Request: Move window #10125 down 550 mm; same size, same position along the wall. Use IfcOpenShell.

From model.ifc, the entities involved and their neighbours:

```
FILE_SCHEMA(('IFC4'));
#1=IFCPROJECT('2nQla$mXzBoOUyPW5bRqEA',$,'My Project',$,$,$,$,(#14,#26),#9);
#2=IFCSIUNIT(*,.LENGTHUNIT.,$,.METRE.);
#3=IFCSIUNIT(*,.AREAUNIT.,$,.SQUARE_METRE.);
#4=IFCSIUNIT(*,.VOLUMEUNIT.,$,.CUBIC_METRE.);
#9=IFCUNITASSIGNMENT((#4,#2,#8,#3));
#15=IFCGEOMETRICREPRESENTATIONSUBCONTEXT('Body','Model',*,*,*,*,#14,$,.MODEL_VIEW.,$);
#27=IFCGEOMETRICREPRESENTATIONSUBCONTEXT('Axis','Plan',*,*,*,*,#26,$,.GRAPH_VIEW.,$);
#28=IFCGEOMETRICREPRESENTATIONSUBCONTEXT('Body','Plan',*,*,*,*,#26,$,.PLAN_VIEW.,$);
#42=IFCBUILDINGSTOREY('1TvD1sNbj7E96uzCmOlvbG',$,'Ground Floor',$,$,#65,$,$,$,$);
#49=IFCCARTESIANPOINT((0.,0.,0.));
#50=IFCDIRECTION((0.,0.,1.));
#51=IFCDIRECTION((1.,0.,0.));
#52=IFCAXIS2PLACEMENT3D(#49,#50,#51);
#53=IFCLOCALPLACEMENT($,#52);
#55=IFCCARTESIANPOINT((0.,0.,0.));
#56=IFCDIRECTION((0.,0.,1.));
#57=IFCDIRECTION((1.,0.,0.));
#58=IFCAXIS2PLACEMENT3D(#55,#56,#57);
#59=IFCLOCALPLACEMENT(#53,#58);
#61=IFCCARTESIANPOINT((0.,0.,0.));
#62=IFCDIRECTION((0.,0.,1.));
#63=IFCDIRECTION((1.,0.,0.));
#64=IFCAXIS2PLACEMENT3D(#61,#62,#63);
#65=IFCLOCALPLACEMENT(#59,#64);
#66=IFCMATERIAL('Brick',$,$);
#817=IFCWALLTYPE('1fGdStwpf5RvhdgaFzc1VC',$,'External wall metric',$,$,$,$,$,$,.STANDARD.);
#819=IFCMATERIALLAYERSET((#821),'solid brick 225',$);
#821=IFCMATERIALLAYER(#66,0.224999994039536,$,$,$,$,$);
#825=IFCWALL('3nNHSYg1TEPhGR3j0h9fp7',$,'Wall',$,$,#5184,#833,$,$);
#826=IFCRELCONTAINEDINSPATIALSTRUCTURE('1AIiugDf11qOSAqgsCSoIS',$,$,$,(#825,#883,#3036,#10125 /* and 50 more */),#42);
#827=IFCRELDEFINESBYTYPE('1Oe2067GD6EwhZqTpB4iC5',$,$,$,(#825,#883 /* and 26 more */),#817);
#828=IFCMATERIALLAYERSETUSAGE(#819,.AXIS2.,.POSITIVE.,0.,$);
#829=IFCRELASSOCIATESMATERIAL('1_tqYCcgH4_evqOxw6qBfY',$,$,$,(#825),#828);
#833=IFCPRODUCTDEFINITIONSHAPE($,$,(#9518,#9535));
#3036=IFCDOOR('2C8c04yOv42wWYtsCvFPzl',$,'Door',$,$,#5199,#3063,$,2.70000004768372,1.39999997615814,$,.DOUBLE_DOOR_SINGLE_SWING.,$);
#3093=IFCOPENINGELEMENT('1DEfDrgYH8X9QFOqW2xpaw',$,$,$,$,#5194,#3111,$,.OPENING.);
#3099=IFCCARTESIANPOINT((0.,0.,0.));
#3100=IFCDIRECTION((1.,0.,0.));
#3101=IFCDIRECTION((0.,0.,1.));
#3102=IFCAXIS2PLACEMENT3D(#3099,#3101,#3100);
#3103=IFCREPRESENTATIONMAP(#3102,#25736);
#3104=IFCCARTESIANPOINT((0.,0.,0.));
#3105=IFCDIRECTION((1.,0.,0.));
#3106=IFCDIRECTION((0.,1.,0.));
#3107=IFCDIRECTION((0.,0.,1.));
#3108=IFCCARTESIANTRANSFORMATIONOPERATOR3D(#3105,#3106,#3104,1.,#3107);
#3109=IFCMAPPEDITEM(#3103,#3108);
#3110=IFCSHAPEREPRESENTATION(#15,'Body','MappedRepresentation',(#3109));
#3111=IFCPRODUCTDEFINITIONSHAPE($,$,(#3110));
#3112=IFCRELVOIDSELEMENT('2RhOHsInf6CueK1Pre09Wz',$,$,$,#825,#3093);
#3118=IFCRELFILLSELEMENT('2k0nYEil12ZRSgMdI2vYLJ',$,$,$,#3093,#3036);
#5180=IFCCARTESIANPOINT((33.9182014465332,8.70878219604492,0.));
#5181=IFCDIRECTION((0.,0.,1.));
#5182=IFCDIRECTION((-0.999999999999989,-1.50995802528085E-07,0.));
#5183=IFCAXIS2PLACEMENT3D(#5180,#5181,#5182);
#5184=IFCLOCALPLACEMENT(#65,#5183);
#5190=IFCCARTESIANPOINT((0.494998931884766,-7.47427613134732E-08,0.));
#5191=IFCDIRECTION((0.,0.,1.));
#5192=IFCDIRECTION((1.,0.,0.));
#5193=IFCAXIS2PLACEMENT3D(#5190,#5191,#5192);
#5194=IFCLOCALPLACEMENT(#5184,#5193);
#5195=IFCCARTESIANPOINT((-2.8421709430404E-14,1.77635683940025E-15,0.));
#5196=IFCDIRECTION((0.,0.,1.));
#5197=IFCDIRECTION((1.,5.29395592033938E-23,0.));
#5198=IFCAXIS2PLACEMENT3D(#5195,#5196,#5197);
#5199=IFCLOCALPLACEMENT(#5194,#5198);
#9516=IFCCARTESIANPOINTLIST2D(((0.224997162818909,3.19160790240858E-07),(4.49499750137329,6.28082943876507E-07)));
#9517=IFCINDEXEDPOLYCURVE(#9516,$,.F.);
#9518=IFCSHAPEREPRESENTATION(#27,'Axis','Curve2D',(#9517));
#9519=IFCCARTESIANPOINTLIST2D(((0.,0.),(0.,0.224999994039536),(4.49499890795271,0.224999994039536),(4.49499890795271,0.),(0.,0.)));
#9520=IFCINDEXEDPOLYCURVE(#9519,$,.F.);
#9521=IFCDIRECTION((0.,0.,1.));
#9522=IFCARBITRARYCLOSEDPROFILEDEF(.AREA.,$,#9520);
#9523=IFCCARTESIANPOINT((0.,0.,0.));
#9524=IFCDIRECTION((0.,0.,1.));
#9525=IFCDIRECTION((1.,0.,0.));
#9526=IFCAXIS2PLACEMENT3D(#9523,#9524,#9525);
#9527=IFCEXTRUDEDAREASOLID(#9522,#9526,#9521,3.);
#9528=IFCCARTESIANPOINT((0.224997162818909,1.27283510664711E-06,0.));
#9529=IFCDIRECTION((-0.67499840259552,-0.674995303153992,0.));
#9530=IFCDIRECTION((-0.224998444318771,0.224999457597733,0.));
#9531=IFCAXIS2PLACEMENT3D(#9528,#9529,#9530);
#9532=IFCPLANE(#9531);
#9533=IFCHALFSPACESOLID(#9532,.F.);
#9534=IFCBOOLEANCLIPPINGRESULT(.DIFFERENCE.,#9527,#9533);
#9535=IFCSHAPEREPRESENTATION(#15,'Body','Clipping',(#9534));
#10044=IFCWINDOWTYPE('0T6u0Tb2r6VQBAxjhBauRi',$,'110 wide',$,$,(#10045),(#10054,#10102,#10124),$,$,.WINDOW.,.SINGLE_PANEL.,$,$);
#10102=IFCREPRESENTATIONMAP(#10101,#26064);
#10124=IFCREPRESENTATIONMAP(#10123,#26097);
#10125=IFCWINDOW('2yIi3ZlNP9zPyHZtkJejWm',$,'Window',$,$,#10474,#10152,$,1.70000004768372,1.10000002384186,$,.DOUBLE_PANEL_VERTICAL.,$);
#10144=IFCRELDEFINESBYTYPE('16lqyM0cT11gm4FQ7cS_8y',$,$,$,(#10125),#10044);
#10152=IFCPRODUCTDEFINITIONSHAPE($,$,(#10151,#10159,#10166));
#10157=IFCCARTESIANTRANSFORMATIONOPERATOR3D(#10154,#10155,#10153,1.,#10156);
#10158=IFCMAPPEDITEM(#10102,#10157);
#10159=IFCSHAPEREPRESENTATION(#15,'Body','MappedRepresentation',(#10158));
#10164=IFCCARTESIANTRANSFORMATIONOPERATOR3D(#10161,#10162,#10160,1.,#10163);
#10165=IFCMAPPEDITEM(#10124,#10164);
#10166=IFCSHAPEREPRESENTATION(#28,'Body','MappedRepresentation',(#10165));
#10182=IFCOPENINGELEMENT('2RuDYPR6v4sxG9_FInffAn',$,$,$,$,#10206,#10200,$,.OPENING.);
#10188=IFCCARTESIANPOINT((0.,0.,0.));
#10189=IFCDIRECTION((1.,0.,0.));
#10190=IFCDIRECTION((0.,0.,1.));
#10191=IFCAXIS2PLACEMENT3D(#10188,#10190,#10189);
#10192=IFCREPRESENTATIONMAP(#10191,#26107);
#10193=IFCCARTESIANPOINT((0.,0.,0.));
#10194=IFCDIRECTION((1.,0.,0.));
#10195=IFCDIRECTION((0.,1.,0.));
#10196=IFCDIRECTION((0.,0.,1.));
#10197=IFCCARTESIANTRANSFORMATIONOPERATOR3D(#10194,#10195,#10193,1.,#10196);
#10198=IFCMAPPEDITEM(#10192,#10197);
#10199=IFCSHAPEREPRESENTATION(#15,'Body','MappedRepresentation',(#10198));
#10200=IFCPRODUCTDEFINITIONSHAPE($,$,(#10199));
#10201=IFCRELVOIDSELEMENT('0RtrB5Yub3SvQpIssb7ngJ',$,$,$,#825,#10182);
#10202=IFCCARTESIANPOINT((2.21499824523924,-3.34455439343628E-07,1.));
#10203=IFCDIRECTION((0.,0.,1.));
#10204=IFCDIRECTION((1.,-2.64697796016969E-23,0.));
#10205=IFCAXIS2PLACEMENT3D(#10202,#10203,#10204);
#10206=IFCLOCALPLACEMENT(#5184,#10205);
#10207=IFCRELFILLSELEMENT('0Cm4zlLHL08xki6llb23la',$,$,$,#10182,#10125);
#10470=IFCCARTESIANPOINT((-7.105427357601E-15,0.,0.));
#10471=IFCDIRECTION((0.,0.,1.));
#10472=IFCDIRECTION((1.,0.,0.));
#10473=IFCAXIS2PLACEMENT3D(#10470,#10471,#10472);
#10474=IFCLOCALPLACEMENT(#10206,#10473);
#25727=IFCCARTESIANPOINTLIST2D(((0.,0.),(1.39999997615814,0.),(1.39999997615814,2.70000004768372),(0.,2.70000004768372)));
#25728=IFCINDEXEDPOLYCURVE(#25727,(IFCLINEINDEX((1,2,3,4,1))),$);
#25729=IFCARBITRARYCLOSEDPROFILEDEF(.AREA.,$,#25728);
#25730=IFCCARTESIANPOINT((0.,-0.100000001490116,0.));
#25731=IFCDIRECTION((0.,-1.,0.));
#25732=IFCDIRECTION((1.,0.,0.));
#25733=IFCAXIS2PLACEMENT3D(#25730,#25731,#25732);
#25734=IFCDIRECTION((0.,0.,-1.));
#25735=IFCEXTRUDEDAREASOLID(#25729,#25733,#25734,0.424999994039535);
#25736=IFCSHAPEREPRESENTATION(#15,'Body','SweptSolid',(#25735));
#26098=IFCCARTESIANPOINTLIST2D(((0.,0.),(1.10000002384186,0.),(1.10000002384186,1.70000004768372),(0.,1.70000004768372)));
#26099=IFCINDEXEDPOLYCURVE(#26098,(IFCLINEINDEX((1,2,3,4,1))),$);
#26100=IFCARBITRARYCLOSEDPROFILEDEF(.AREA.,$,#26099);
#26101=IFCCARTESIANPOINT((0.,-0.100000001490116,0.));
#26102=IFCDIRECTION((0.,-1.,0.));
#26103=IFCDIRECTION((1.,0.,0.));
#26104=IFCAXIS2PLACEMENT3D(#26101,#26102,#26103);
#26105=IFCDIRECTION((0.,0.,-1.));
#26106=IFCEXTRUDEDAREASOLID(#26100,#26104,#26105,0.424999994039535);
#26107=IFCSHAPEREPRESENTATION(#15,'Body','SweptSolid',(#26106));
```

```python
import numpy as np
import ifcopenshell
import ifcopenshell.api.geometry
import ifcopenshell.util.placement
import ifcopenshell.util.unit

model = ifcopenshell.open("model.ifc")
unit_scale = ifcopenshell.util.unit.calculate_unit_scale(model)

window = model.by_id(10125)
opening = window.FillsVoids[0].RelatingOpeningElement
dz = -0.55 / unit_scale

shift = np.array([0.0, 0.0, dz])
# The window is placed relative to its opening, so it follows when the opening moves.
matrix = ifcopenshell.util.placement.get_local_placement(opening.ObjectPlacement)
matrix[:3, 3] += shift
ifcopenshell.api.geometry.edit_object_placement(
    model, product=opening, matrix=matrix, is_si=False, should_transform_children=True
)

print(f"moved by {dz * unit_scale:+.3f} m")

model.write("model-out.ifc")
```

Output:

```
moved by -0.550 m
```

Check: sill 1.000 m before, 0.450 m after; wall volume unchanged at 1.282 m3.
